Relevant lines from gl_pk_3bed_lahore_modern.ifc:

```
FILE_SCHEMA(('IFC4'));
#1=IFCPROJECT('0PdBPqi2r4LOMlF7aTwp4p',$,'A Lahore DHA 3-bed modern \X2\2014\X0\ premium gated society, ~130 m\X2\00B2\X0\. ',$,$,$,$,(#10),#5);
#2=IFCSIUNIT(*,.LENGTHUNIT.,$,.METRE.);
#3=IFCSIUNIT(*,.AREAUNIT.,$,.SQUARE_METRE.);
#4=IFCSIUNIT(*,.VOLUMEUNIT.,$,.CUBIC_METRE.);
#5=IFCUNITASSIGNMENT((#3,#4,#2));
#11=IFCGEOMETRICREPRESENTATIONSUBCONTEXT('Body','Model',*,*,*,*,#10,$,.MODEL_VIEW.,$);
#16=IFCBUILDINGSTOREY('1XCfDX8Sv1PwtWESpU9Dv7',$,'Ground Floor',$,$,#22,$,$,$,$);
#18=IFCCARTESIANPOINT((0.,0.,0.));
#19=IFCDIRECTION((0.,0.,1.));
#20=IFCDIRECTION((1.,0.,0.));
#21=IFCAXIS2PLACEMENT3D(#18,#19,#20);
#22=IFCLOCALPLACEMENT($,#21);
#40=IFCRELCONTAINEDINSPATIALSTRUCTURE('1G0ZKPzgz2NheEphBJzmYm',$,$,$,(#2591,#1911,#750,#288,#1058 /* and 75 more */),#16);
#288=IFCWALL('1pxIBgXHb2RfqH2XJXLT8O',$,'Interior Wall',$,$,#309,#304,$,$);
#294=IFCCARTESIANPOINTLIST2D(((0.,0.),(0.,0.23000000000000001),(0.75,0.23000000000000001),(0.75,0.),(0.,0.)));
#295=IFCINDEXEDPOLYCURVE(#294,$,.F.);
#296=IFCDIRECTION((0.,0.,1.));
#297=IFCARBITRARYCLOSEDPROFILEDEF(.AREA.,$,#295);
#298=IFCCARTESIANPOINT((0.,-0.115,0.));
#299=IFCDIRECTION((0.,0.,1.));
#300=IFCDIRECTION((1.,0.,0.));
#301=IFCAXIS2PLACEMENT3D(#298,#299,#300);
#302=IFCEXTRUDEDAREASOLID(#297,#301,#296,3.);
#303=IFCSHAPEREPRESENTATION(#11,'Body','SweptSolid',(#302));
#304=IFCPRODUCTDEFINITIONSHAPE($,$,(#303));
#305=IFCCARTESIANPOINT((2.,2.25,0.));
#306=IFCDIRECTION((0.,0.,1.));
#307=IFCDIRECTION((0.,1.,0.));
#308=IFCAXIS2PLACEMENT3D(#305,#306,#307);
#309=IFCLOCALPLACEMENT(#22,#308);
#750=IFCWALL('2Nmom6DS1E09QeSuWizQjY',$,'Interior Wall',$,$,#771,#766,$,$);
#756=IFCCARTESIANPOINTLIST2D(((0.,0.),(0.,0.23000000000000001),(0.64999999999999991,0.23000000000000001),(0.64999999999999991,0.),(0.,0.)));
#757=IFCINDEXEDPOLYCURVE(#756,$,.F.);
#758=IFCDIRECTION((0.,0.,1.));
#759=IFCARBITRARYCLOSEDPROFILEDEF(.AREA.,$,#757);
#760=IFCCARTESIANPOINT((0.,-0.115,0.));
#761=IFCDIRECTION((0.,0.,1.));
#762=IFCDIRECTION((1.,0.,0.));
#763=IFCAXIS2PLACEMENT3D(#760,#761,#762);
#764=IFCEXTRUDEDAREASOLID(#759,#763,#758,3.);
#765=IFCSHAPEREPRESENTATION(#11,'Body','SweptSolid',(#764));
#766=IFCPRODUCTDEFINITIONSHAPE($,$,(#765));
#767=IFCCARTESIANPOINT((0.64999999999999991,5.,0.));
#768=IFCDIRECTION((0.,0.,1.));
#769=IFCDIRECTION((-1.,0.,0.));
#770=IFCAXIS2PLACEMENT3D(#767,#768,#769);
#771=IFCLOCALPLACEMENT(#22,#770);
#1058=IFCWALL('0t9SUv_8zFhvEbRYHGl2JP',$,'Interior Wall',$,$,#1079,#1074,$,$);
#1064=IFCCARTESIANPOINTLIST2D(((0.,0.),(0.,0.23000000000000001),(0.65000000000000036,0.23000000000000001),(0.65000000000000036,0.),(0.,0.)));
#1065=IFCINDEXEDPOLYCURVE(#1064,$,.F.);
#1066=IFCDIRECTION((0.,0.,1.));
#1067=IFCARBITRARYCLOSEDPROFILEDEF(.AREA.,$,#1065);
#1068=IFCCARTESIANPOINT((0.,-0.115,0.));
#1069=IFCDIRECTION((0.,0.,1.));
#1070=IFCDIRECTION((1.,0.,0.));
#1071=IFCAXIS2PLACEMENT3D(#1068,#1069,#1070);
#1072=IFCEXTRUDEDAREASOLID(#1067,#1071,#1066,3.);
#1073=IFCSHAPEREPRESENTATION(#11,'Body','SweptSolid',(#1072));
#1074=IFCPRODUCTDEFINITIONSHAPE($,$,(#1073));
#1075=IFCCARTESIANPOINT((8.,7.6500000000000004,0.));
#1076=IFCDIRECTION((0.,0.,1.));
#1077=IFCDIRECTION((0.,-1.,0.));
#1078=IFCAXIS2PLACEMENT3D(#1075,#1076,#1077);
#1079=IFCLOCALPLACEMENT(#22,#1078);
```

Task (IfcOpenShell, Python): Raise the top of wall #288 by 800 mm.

```python
import ifcopenshell
import ifcopenshell.geom
import ifcopenshell.util.representation
import ifcopenshell.util.shape
import ifcopenshell.util.unit

model = ifcopenshell.open("gl_pk_3bed_lahore_modern.ifc")
unit_scale = ifcopenshell.util.unit.calculate_unit_scale(model)
settings = ifcopenshell.geom.settings()


def volume(element):
    """Net volume in cubic metres, openings subtracted."""
    shape = ifcopenshell.geom.create_shape(settings, element)
    return ifcopenshell.util.shape.get_volume(shape.geometry)


wall = model.by_guid("1pxIBgXHb2RfqH2XJXLT8O")
before = volume(wall)

body = ifcopenshell.util.representation.get_representation(wall, "Model", "Body")
solid = body.Items[0]
old_height = solid.Depth
solid.Depth += 0.8 / unit_scale
after = volume(wall)

print(f"height {old_height:g} -> {solid.Depth:g}, volume {before:.3f} -> {after:.3f} m3")

model.write("gl_pk_3bed_lahore_modern-out.ifc")
```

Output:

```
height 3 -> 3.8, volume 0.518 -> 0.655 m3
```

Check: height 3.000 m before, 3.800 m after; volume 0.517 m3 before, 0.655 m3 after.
